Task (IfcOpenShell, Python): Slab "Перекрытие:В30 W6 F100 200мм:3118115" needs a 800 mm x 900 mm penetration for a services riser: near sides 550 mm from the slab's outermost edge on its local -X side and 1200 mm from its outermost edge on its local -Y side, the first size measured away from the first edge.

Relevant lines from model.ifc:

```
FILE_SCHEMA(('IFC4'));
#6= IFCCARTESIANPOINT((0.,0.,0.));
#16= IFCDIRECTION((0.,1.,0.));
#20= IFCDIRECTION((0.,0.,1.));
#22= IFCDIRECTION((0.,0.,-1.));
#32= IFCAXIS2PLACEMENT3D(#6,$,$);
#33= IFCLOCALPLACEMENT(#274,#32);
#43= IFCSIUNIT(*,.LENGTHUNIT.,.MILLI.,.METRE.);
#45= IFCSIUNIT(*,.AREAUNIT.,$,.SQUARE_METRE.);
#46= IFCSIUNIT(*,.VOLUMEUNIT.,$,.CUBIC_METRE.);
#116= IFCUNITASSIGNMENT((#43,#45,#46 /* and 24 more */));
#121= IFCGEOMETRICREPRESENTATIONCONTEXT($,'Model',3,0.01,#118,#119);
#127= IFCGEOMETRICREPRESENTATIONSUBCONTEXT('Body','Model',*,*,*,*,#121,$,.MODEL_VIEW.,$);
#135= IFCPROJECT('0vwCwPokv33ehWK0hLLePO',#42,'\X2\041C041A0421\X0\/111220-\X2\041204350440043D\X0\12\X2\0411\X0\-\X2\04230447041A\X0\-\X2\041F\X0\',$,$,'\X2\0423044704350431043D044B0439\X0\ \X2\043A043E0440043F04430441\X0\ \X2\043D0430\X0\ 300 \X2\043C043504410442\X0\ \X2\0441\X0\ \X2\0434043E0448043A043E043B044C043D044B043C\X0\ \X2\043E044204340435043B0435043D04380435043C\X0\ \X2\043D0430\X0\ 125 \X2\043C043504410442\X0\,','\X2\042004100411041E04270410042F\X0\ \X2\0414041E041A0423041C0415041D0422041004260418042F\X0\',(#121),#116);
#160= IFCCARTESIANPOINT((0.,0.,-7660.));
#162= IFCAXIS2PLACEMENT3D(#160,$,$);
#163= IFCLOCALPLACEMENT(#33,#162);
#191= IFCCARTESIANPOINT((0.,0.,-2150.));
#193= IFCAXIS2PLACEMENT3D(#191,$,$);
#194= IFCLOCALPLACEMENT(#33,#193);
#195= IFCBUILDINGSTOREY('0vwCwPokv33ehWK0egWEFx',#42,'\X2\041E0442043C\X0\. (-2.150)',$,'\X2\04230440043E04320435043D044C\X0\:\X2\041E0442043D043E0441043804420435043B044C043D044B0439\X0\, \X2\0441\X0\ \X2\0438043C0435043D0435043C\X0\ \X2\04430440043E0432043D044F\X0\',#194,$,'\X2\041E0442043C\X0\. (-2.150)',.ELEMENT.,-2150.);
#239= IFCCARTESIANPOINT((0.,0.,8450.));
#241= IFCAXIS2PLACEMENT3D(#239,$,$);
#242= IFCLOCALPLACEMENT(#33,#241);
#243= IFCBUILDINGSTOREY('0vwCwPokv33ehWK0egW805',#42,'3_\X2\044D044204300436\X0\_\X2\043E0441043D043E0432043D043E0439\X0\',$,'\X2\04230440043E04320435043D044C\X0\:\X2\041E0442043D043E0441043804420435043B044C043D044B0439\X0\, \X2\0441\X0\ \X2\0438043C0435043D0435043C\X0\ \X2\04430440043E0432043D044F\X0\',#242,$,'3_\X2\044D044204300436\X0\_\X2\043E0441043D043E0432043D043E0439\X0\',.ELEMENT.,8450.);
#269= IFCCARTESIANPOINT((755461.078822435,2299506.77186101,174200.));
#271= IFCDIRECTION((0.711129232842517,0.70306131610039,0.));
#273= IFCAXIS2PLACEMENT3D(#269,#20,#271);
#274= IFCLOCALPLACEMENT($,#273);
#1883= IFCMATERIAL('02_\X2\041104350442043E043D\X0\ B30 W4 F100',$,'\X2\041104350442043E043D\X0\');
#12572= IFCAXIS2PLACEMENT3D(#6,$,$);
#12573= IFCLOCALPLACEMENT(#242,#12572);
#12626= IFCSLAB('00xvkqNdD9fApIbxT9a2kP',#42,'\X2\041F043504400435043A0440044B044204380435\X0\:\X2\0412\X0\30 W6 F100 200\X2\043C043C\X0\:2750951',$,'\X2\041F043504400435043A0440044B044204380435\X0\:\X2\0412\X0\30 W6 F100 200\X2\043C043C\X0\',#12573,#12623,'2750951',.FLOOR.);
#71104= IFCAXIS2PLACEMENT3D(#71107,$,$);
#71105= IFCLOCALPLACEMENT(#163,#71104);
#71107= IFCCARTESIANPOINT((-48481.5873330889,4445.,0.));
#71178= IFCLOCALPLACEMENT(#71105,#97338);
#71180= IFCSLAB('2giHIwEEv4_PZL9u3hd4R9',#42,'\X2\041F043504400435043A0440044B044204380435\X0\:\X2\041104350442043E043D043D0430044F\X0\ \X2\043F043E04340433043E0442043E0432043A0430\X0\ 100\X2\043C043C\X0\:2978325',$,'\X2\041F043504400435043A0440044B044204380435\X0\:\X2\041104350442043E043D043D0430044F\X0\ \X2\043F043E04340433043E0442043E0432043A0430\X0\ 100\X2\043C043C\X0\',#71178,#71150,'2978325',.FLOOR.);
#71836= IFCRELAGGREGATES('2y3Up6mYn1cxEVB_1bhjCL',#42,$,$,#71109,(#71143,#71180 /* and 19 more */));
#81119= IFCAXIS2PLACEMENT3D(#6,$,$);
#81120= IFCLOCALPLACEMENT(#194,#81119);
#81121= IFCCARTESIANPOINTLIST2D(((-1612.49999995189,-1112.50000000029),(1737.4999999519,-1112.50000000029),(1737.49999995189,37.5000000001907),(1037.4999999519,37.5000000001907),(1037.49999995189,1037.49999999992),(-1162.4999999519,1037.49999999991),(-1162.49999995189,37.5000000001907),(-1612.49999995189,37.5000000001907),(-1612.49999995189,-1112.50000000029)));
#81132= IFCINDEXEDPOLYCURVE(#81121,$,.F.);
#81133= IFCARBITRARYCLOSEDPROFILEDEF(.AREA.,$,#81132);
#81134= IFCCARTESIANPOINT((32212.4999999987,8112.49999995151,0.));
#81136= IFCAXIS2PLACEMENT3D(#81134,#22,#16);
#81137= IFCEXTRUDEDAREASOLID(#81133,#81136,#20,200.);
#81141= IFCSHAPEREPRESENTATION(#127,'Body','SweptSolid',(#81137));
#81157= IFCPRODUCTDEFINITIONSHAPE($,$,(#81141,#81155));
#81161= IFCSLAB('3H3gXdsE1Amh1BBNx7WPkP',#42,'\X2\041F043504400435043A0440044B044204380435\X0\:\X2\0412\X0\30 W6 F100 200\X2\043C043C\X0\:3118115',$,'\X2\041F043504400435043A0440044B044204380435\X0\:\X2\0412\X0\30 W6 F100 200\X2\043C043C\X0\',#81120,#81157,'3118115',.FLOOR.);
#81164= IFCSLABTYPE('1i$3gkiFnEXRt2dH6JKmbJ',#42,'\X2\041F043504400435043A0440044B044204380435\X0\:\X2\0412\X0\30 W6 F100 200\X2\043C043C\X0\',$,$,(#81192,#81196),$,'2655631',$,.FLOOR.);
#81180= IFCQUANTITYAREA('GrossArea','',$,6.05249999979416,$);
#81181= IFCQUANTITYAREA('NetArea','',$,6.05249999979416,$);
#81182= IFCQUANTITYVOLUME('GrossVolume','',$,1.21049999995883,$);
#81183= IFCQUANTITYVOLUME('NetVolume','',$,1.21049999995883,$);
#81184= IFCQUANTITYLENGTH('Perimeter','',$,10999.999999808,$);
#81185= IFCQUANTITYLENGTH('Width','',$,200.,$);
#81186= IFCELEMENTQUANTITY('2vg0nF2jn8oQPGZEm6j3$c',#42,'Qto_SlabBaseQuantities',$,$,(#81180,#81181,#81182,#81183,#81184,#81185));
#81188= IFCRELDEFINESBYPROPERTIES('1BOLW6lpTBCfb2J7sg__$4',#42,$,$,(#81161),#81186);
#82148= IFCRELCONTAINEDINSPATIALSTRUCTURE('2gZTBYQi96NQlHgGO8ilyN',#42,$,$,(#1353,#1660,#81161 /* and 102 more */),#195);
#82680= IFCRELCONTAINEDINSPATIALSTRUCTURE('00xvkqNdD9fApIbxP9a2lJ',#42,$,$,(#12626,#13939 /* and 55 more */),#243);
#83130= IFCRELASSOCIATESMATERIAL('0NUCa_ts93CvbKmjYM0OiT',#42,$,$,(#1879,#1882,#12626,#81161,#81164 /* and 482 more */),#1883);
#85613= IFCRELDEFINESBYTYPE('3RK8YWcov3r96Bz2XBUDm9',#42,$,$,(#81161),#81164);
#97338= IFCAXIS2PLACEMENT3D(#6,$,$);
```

```python
import numpy as np
import ifcopenshell
import ifcopenshell.api.feature
import ifcopenshell.api.geometry
import ifcopenshell.api.pset
import ifcopenshell.api.root
import ifcopenshell.geom
import ifcopenshell.util.element
import ifcopenshell.util.placement
import ifcopenshell.util.representation
import ifcopenshell.util.shape
import ifcopenshell.util.unit

model = ifcopenshell.open("model.ifc")
unit_scale = ifcopenshell.util.unit.calculate_unit_scale(model)
area_scale = ifcopenshell.util.unit.calculate_unit_scale(model, "AREAUNIT")
volume_scale = ifcopenshell.util.unit.calculate_unit_scale(model, "VOLUMEUNIT")
settings = ifcopenshell.geom.settings()


def volume(element):
    """Net volume in cubic metres, openings subtracted."""
    shape = ifcopenshell.geom.create_shape(settings, element)
    return ifcopenshell.util.shape.get_volume(shape.geometry)


slab = model.by_id(81161)
before = volume(slab)

# Extent in the slab's own axes, in metres. The edges named are its -X and -Y sides.
slab_shape = ifcopenshell.geom.create_shape(settings, slab)
vertices = ifcopenshell.util.shape.get_vertices(slab_shape.geometry)
x_min, y_min, bottom = vertices.min(axis=0)
top = vertices[:, 2].max()

opening = ifcopenshell.api.root.create_entity(model, ifc_class="IfcOpeningElement", name="Services riser opening", predefined_type="OPENING")
context = ifcopenshell.util.representation.get_context(model, "Model", "Body", "MODEL_VIEW")
width, depth = 0.8, 0.9
outline = [(0.0, 0.0), (width, 0.0), (width, depth), (0.0, depth), (0.0, 0.0)]
# Overshoot both faces by 50 mm so the cut is clean.
shape = ifcopenshell.api.geometry.add_slab_representation(
    model, context=context, depth=top - bottom + 0.1, polyline=outline
)
ifcopenshell.api.geometry.assign_representation(model, product=opening, representation=shape)

matrix = ifcopenshell.util.placement.get_local_placement(slab.ObjectPlacement)
matrix[:, 3] = matrix @ np.append(np.array([x_min + 0.55, y_min + 1.2, bottom - 0.05]) / unit_scale, 1.0)
ifcopenshell.api.geometry.edit_object_placement(model, product=opening, matrix=matrix, is_si=False)
ifcopenshell.api.feature.add_feature(model, feature=opening, element=slab)

after = volume(slab)

# Update the slab's stored quantities.
qto = model.by_id(ifcopenshell.util.element.get_pset(slab, "Qto_SlabBaseQuantities", should_inherit=False)["id"])
ifcopenshell.api.pset.edit_qto(model, qto=qto, properties={
    "NetArea": after / (top - bottom) / area_scale,
    "NetVolume": after / volume_scale,
})

print(f"slab volume {before:.3f} -> {after:.3f} m3")

model.write("model_v2.ifc")
```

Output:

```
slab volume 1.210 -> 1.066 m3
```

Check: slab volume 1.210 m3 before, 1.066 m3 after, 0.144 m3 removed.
